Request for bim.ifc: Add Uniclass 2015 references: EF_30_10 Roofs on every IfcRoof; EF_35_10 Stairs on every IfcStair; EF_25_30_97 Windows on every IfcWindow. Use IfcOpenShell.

First a look at what the model holds.

```python
import ifcopenshell

model = ifcopenshell.open("bim.ifc")
print(model.schema)
print("classifications:", [c.Name for c in model.by_type("IfcClassification")])
for ifc_class in ("IfcDoor", "IfcRoof", "IfcStair", "IfcWall", "IfcWindow"):
    print(ifc_class, len(model.by_type(ifc_class)))
```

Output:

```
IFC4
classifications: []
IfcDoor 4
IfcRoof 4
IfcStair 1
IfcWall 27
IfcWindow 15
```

```python
import ifcopenshell
import ifcopenshell.api.classification

model = ifcopenshell.open("bim.ifc")

system = ifcopenshell.api.classification.add_classification(model, classification="Uniclass 2015")

codes = {
    "IfcRoof": ("EF_30_10", "Roofs"),
    "IfcStair": ("EF_35_10", "Stairs"),
    "IfcWindow": ("EF_25_30_97", "Windows"),
}
for ifc_class, (code, name) in codes.items():
    products = model.by_type(ifc_class)
    ifcopenshell.api.classification.add_reference(
        model, products=products, classification=system, identification=code, name=name
    )
    print(code, len(products))

model.write("bim_updated.ifc")
```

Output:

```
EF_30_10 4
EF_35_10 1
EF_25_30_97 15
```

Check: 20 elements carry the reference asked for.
